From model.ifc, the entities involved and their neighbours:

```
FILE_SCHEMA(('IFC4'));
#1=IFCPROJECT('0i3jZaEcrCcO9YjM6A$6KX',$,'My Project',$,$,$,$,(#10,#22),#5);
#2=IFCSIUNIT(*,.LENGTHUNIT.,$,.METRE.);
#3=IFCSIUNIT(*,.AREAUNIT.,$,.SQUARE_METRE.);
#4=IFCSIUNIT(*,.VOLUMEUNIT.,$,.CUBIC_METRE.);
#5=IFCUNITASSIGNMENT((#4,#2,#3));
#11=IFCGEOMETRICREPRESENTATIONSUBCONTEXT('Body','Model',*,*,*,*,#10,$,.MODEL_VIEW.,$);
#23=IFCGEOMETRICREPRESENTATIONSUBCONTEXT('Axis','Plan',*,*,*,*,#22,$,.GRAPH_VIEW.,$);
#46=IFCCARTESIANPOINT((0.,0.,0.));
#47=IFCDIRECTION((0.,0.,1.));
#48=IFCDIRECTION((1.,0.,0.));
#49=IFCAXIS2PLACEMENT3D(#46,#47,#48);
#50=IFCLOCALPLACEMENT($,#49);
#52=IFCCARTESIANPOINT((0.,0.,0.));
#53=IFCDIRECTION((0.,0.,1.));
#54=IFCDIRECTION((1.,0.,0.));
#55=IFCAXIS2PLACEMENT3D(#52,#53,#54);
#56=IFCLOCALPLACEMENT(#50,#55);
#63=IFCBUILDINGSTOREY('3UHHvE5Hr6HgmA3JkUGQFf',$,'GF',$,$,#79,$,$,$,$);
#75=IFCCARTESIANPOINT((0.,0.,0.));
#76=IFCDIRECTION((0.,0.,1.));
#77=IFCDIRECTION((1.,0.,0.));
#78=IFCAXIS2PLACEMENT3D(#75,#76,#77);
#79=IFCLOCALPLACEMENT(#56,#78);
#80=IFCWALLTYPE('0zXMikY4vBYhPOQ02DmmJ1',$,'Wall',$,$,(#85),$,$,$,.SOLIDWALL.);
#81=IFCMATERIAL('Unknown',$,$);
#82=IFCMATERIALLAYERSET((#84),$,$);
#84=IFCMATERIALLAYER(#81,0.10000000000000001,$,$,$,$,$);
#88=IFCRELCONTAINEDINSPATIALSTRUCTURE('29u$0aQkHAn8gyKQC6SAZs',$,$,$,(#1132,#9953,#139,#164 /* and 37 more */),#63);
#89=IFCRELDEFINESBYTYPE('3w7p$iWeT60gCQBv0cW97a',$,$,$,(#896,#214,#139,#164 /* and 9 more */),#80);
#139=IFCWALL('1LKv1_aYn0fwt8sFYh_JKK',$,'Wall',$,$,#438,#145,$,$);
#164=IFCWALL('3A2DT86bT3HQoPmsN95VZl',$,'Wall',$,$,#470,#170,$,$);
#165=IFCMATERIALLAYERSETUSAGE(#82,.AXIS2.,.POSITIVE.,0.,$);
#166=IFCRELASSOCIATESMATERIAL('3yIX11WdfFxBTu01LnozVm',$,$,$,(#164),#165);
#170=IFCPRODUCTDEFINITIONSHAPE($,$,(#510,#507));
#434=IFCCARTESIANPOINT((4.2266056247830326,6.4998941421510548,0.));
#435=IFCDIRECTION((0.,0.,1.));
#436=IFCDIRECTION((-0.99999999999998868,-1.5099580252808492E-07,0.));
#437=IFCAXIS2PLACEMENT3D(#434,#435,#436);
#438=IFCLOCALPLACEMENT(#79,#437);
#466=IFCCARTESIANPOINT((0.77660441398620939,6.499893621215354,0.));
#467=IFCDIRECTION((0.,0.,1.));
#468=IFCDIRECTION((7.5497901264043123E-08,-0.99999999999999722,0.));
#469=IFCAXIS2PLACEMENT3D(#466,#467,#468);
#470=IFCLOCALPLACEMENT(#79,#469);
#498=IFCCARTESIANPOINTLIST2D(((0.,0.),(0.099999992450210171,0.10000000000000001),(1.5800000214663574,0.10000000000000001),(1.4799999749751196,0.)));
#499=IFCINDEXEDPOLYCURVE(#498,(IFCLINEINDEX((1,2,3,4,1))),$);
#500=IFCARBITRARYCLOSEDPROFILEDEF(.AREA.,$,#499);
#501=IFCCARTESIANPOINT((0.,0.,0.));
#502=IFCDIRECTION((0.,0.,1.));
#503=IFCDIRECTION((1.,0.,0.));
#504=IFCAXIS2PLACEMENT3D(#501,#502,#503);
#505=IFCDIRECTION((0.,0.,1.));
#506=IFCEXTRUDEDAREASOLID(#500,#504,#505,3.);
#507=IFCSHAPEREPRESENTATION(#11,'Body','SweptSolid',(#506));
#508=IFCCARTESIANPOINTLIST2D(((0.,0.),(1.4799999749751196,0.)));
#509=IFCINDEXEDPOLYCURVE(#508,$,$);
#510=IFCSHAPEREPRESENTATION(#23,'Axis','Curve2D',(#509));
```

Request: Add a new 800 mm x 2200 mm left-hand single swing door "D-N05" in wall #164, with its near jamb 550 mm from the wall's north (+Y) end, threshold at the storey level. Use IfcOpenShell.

```python
import numpy as np
import ifcopenshell
import ifcopenshell.api.feature
import ifcopenshell.api.geometry
import ifcopenshell.api.root
import ifcopenshell.api.spatial
import ifcopenshell.geom
import ifcopenshell.util.element
import ifcopenshell.util.placement
import ifcopenshell.util.representation
import ifcopenshell.util.shape
import ifcopenshell.util.unit

model = ifcopenshell.open("model.ifc")
unit_scale = ifcopenshell.util.unit.calculate_unit_scale(model)
settings = ifcopenshell.geom.settings()


def volume(element):
    """Net volume in cubic metres, openings subtracted."""
    shape = ifcopenshell.geom.create_shape(settings, element)
    return ifcopenshell.util.shape.get_volume(shape.geometry)


wall = model.by_guid("3A2DT86bT3HQoPmsN95VZl")
storey = ifcopenshell.util.element.get_container(wall, ifc_class="IfcBuildingStorey")
context = ifcopenshell.util.representation.get_context(model, "Model", "Body", "MODEL_VIEW")
before = volume(wall)

width, height, from_end, sill = 0.8, 2.2, 0.55, 0.0  # metres

# The wall runs along its own X axis, and the end named is its -X end.
wall_shape = ifcopenshell.geom.create_shape(settings, wall)
x, y, z = ifcopenshell.util.shape.get_vertices(wall_shape.geometry).T
start = x.min() + from_end
face, thickness = float(y.min()), float(y.max() - y.min())
wall_matrix = ifcopenshell.util.placement.get_local_placement(wall.ObjectPlacement)
level = ifcopenshell.util.placement.get_local_placement(storey.ObjectPlacement)[2, 3]


def in_wall(x, y):
    """Placement at x, y metres in the wall's axes, at sill height."""
    matrix = wall_matrix.copy()
    matrix[:, 3] = wall_matrix @ np.array([x / unit_scale, y / unit_scale, 0.0, 1.0])
    matrix[2, 3] = level + sill / unit_scale
    return matrix


# Opening: a box that overshoots both wall faces by 50 mm.
opening = ifcopenshell.api.root.create_entity(model, ifc_class="IfcOpeningElement", predefined_type="OPENING")
box = ifcopenshell.api.geometry.add_wall_representation(
    model, context=context, length=width, height=height, thickness=thickness + 0.1
)
ifcopenshell.api.geometry.assign_representation(model, product=opening, representation=box)
ifcopenshell.api.geometry.edit_object_placement(model, product=opening, matrix=in_wall(start, face - 0.05), is_si=False)
ifcopenshell.api.feature.add_feature(model, feature=opening, element=wall)

door = ifcopenshell.api.root.create_entity(model, ifc_class="IfcDoor", name="D-N05", predefined_type="DOOR")
door.OverallWidth, door.OverallHeight = width / unit_scale, height / unit_scale
door.OperationType = "SINGLE_SWING_LEFT"
body = ifcopenshell.api.geometry.add_door_representation(
    model,
    context=context,
    overall_width=door.OverallWidth,
    overall_height=door.OverallHeight,
    operation_type="SINGLE_SWING_LEFT",
    lining_properties={"LiningDepth": thickness / unit_scale, "ThresholdDepth": thickness / unit_scale},
)
ifcopenshell.api.geometry.assign_representation(model, product=door, representation=body)
ifcopenshell.api.spatial.assign_container(model, products=[door], relating_structure=storey)
ifcopenshell.api.feature.add_filling(model, opening=opening, element=door)

# The lining spans the wall, so the door starts at the wall face.
ifcopenshell.api.geometry.edit_object_placement(model, product=door, matrix=in_wall(start, face), is_si=False)

after = volume(wall)

print(f"wall volume {before:.3f} -> {after:.3f} m3")

model.write("model-out.ifc")
```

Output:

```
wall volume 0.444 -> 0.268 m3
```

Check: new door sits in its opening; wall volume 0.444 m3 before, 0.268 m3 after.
